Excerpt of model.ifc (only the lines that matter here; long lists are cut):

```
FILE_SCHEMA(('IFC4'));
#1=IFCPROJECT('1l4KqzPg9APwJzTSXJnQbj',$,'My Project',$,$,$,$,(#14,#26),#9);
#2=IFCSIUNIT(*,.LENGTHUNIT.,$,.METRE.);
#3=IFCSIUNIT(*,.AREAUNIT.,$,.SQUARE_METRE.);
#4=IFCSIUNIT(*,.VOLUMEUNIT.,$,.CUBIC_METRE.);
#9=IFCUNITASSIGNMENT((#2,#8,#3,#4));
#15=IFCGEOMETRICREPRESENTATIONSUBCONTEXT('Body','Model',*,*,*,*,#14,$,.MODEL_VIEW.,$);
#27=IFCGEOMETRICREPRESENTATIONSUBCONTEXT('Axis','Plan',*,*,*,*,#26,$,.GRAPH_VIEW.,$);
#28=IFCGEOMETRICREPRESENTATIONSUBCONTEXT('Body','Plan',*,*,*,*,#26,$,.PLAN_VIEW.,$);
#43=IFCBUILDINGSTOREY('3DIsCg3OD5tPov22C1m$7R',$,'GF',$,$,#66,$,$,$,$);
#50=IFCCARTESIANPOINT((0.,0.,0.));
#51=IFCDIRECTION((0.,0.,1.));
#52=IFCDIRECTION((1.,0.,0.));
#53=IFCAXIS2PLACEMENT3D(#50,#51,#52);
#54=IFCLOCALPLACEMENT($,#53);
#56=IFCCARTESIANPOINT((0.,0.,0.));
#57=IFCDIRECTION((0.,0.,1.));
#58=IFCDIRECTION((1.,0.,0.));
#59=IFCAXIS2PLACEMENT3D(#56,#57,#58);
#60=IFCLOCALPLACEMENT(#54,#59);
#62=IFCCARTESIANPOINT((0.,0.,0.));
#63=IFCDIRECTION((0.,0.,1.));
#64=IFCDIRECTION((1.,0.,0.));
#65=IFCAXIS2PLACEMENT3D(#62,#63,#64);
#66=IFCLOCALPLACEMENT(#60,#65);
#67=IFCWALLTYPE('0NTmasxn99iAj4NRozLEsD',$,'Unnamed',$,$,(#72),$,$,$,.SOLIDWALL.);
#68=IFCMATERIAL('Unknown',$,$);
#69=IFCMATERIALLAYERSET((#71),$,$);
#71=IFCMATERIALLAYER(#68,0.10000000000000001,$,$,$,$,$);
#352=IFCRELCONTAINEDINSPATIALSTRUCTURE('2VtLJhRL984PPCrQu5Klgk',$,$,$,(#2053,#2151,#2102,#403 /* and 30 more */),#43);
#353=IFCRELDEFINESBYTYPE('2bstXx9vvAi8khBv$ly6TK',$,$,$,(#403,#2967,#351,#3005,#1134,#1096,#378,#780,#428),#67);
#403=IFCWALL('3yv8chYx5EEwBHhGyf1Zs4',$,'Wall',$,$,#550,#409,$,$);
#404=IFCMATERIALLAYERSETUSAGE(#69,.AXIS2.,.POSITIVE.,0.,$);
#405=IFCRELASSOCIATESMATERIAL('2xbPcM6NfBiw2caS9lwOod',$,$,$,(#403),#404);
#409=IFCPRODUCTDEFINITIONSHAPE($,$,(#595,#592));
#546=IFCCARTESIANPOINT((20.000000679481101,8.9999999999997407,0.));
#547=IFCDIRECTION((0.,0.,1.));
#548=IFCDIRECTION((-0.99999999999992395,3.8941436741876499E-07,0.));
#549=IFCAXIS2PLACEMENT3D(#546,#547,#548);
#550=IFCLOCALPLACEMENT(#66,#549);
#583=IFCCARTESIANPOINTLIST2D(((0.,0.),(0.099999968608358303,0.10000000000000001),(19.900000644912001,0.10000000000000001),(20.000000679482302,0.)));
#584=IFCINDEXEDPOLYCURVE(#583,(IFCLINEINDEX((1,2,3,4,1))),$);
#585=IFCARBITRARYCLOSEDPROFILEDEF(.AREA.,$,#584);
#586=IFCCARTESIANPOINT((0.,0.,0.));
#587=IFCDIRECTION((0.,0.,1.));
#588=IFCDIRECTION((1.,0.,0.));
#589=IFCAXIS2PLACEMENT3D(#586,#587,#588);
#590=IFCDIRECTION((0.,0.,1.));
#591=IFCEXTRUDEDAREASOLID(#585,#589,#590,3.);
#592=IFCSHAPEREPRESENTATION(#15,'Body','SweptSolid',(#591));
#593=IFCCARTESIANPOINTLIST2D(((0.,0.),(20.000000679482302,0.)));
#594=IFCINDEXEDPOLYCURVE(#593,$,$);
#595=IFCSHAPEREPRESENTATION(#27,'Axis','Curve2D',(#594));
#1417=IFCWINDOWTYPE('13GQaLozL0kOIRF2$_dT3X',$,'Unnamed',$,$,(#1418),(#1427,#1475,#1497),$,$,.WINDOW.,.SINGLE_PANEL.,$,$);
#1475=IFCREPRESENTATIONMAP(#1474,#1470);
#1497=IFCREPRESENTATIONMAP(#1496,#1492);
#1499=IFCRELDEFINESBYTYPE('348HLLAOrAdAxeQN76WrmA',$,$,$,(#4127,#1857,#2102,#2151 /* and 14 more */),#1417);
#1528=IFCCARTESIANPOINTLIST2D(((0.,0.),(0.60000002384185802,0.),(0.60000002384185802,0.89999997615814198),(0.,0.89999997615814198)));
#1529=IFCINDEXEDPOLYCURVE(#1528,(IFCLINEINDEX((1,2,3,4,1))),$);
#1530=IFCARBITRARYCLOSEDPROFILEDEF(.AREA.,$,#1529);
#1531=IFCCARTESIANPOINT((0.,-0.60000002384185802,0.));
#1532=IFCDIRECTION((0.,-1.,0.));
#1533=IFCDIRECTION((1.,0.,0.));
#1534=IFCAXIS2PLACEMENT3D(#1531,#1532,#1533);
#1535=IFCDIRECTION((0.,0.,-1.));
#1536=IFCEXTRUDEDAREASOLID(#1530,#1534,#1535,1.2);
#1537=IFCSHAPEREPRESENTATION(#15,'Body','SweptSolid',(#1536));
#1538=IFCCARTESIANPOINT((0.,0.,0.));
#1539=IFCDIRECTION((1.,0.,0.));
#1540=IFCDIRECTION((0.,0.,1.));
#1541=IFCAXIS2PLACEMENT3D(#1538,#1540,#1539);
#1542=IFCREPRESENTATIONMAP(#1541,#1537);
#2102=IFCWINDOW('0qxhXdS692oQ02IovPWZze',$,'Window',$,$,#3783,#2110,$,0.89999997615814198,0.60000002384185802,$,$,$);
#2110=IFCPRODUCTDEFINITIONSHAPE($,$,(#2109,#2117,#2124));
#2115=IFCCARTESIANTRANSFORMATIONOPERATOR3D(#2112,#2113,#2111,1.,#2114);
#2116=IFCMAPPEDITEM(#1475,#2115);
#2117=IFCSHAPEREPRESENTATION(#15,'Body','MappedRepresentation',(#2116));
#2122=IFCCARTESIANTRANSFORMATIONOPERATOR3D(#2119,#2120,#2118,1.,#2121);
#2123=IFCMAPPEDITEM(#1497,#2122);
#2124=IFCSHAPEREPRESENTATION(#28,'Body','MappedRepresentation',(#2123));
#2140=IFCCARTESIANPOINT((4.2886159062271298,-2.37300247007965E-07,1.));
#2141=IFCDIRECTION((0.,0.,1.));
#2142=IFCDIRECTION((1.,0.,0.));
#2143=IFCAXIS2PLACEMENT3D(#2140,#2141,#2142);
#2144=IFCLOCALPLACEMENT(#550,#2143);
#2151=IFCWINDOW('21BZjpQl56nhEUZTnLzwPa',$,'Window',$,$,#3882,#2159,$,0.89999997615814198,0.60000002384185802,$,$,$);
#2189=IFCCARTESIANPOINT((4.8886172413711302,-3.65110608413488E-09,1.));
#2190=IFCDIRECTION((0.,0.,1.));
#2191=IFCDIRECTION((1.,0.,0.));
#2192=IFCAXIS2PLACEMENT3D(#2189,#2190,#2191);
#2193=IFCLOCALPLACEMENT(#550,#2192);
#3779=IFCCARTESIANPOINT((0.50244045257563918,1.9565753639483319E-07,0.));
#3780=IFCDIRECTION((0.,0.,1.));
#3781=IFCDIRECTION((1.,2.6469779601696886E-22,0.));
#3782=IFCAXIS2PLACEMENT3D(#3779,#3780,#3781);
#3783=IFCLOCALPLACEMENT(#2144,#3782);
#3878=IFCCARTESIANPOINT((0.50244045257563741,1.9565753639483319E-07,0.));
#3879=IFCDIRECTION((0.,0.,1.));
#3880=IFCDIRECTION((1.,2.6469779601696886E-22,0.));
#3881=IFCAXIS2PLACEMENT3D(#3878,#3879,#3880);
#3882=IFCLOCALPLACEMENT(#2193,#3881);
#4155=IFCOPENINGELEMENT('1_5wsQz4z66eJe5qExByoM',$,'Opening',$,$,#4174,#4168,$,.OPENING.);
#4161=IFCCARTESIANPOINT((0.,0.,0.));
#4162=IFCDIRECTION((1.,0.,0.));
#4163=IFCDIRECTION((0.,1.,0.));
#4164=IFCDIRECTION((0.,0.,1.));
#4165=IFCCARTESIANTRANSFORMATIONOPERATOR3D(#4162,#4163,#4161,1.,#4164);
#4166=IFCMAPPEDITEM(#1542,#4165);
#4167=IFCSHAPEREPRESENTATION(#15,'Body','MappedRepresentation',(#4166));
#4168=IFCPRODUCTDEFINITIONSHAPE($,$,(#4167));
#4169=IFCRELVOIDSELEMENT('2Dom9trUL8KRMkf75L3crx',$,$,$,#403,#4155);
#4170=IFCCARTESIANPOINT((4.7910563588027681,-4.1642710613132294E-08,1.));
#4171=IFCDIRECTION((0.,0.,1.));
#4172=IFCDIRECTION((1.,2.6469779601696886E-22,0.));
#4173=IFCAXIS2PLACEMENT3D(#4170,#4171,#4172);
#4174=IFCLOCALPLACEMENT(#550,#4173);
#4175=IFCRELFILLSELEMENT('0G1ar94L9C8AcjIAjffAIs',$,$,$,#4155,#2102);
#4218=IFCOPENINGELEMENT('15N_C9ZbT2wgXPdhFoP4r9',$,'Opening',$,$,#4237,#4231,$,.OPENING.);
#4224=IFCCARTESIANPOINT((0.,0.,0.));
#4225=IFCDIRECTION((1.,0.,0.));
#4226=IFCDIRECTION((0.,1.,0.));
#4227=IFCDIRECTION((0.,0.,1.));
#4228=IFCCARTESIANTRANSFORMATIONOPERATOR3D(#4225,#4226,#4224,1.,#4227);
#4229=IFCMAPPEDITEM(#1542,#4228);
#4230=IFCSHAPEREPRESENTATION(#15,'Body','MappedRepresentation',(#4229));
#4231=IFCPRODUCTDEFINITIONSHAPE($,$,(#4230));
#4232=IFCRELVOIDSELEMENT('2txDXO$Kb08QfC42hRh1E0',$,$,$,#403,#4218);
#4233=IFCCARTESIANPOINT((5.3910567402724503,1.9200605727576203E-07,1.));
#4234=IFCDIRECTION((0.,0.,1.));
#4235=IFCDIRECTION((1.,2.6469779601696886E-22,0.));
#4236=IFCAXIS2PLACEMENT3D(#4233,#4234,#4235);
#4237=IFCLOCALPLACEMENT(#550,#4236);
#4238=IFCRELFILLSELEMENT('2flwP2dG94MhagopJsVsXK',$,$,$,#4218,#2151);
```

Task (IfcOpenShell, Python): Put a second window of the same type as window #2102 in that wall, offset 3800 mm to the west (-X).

```python
import ifcopenshell
import ifcopenshell.api.feature
import ifcopenshell.api.geometry
import ifcopenshell.api.root
import ifcopenshell.geom
import ifcopenshell.util.element
import ifcopenshell.util.placement
import ifcopenshell.util.shape

model = ifcopenshell.open("model.ifc")
settings = ifcopenshell.geom.settings()


def volume(element):
    """Net volume in cubic metres, openings subtracted."""
    shape = ifcopenshell.geom.create_shape(settings, element)
    return ifcopenshell.util.shape.get_volume(shape.geometry)


window = model.by_guid("0qxhXdS692oQ02IovPWZze")
opening = window.FillsVoids[0].RelatingOpeningElement
wall = opening.VoidsElements[0].RelatingBuildingElement
before = volume(wall)
shift = ifcopenshell.util.placement.get_local_placement(wall.ObjectPlacement)[:3, 0] * 3.8

# copy_class copies the void relationship, type, container and properties, but no geometry.
new_opening = ifcopenshell.api.root.copy_class(model, product=opening)
new_opening.Representation = ifcopenshell.util.element.copy_deep(
    model, opening.Representation, exclude=["IfcGeometricRepresentationContext", "IfcRepresentationMap"]
)
new_window = ifcopenshell.api.root.copy_class(model, product=window)
new_window.Representation = ifcopenshell.util.element.copy_deep(
    model, window.Representation, exclude=["IfcGeometricRepresentationContext", "IfcRepresentationMap"]
)
ifcopenshell.api.feature.add_filling(model, opening=new_opening, element=new_window)

for old, new in ((opening, new_opening), (window, new_window)):
    matrix = ifcopenshell.util.placement.get_local_placement(old.ObjectPlacement)
    matrix[:3, 3] += shift
    ifcopenshell.api.geometry.edit_object_placement(model, product=new, matrix=matrix, is_si=False)

after = volume(wall)

print(f"wall volume {before:.3f} -> {after:.3f} m3")

model.write("model_edited.ifc")
```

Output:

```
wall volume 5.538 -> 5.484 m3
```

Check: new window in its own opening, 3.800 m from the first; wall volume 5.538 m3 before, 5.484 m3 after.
